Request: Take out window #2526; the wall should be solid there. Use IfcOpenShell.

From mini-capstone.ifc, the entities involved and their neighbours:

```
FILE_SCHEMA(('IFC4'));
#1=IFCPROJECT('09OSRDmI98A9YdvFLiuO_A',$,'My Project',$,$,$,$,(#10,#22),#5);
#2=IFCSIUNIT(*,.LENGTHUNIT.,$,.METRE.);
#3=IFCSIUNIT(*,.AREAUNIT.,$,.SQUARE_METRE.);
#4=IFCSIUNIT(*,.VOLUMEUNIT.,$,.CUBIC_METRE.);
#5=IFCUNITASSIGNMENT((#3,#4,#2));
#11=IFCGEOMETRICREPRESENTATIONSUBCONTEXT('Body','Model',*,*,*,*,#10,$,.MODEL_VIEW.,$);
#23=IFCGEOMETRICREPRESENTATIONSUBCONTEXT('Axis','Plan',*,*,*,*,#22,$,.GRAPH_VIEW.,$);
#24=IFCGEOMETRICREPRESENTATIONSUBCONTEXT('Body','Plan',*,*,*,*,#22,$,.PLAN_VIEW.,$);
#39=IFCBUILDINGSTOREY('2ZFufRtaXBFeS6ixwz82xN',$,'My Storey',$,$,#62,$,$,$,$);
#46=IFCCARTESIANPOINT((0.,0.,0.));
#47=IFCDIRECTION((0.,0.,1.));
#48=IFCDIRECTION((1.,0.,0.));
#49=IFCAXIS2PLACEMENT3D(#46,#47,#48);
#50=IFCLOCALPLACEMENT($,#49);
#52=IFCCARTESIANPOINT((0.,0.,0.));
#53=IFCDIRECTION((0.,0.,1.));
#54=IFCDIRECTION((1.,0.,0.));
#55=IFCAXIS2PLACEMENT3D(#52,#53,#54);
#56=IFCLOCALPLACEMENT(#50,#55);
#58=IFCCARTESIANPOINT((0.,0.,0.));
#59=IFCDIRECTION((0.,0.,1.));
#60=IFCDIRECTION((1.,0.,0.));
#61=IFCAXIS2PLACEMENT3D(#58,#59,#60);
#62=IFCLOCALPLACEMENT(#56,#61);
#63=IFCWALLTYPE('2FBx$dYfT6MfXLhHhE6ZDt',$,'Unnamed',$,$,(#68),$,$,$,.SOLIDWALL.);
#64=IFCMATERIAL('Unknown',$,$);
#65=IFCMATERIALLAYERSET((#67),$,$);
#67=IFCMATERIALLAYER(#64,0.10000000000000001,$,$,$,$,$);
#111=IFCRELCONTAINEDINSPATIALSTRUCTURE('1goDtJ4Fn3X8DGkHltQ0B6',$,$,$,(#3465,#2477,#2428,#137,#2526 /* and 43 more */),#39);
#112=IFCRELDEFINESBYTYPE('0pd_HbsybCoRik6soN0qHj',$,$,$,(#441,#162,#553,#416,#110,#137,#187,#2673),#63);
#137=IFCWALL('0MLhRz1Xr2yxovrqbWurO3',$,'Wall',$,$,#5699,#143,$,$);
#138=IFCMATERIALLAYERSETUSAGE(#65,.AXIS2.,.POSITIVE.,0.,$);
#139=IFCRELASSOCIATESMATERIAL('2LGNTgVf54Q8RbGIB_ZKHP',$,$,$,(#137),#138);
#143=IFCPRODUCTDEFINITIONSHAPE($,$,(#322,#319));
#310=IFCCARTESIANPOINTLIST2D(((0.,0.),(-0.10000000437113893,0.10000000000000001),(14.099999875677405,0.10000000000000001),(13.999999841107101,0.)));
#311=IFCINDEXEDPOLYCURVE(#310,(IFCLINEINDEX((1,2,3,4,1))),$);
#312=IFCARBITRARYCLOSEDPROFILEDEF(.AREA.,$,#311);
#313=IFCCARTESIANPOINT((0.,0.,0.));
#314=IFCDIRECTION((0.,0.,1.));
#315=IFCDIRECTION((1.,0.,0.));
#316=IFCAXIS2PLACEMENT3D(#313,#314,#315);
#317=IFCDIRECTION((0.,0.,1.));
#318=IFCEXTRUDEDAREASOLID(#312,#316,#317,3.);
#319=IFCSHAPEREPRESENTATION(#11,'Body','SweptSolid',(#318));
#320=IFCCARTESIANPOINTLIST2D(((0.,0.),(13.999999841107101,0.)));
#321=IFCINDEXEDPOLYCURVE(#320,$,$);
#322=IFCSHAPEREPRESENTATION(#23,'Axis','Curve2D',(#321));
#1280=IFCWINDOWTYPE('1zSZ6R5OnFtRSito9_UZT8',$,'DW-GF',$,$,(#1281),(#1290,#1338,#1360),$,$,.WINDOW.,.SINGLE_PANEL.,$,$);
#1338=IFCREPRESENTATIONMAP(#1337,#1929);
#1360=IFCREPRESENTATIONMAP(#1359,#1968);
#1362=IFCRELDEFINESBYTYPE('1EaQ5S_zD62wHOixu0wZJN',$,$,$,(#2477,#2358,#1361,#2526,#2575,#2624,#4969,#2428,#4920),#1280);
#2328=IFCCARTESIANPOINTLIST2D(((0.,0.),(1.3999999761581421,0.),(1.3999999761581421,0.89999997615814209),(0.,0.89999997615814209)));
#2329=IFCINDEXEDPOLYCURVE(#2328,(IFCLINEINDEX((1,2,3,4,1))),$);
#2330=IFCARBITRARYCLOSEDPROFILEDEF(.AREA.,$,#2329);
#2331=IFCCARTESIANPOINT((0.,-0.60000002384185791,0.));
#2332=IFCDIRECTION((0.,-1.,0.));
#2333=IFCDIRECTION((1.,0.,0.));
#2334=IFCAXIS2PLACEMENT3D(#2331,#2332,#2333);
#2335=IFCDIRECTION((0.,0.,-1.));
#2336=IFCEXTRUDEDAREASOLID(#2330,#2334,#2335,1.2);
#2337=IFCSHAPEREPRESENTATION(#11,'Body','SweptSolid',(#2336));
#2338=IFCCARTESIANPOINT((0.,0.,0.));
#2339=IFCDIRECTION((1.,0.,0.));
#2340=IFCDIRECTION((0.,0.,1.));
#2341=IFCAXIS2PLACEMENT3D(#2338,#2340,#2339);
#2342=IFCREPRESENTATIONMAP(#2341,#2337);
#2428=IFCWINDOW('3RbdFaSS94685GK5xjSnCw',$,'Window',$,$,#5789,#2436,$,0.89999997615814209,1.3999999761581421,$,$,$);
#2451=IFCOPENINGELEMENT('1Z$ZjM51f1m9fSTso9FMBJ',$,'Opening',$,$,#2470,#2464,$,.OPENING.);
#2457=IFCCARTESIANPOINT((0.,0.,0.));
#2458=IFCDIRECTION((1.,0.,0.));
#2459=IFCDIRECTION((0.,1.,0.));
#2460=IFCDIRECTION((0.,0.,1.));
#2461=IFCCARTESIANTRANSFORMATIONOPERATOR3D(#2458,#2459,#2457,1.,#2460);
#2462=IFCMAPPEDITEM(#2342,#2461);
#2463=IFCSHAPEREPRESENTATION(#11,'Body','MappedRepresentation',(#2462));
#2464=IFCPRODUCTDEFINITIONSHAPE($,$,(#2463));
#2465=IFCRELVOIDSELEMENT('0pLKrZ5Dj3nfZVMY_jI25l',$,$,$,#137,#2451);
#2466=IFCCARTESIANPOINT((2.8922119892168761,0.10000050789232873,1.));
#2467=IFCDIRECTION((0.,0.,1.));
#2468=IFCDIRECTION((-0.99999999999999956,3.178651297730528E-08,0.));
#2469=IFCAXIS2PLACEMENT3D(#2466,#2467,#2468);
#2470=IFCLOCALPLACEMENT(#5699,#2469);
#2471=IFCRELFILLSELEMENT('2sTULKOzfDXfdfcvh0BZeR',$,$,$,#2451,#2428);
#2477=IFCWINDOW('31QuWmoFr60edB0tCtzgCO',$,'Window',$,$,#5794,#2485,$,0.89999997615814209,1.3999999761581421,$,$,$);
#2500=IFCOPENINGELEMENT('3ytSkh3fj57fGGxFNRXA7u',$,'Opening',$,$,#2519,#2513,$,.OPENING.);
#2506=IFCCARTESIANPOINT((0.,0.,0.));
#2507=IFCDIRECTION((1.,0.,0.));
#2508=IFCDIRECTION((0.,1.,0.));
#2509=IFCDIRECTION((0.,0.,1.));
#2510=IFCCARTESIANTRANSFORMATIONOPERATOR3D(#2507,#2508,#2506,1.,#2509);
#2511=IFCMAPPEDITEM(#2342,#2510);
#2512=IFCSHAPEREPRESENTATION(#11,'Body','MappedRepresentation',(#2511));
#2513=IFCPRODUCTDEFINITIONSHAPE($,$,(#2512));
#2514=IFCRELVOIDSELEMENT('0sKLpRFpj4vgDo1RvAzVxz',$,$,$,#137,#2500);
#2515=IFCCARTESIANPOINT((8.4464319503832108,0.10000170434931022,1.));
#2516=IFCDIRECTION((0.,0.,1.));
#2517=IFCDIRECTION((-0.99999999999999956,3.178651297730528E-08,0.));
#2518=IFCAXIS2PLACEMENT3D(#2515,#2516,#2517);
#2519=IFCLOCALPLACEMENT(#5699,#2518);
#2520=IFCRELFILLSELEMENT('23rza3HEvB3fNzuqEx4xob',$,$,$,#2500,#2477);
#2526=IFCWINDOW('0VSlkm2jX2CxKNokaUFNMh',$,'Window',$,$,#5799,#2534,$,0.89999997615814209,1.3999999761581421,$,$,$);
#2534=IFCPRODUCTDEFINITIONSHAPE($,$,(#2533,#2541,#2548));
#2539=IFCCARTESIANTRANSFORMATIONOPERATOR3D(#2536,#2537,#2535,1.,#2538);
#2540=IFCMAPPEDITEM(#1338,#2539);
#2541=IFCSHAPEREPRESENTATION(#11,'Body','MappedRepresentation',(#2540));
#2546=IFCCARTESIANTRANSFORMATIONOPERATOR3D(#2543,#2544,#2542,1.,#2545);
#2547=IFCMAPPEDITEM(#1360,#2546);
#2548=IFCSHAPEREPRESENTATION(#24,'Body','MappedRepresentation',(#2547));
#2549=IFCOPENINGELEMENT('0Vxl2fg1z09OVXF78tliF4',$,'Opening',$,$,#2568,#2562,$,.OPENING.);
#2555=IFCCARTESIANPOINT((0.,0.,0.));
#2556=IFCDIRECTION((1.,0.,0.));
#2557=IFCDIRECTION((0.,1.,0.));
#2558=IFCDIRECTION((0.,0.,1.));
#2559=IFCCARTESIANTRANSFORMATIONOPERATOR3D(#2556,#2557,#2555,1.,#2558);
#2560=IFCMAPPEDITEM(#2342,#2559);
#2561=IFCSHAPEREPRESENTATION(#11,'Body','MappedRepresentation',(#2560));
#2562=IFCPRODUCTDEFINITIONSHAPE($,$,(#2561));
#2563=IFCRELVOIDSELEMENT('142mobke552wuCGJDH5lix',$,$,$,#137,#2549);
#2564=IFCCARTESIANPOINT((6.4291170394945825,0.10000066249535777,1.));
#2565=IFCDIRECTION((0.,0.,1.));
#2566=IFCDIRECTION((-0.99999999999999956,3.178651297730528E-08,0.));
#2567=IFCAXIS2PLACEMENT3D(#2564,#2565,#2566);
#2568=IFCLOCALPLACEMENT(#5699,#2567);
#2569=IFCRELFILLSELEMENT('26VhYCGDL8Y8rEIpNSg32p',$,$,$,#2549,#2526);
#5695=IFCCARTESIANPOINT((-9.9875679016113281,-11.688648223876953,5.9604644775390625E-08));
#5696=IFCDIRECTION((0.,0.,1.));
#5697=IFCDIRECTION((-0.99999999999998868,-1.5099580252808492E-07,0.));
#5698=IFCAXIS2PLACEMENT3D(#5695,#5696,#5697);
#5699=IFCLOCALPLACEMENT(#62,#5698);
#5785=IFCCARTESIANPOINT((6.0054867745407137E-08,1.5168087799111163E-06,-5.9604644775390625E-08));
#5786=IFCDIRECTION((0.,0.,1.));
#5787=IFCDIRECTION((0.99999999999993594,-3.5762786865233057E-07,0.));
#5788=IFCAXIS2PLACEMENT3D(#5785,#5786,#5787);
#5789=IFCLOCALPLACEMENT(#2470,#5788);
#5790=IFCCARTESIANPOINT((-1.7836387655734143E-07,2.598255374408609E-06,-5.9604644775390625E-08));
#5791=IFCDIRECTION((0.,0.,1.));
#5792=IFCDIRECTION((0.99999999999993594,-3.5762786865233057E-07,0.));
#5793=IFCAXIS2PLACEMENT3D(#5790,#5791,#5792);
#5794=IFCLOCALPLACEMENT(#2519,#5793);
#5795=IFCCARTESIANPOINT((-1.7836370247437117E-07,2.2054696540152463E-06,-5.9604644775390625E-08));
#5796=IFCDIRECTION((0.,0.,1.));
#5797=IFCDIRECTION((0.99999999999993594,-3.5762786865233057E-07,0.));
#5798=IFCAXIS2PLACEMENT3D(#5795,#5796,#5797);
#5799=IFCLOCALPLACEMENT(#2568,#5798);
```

```python
import ifcopenshell
import ifcopenshell.api.feature
import ifcopenshell.api.root
import ifcopenshell.geom
import ifcopenshell.util.shape

model = ifcopenshell.open("mini-capstone.ifc")
settings = ifcopenshell.geom.settings()


def volume(element):
    """Net volume in cubic metres, openings subtracted."""
    shape = ifcopenshell.geom.create_shape(settings, element)
    return ifcopenshell.util.shape.get_volume(shape.geometry)


window = model.by_guid("0VSlkm2jX2CxKNokaUFNMh")
opening = window.FillsVoids[0].RelatingOpeningElement
wall = opening.VoidsElements[0].RelatingBuildingElement
before = volume(wall)

ifcopenshell.api.root.remove_product(model, product=window)
ifcopenshell.api.feature.remove_feature(model, feature=opening)

after = volume(wall)

print(f"wall volume {before:.3f} -> {after:.3f} m3")

model.write("mini-capstone_edited.ifc")
```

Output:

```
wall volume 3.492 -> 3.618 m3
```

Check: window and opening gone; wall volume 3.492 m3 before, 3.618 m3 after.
